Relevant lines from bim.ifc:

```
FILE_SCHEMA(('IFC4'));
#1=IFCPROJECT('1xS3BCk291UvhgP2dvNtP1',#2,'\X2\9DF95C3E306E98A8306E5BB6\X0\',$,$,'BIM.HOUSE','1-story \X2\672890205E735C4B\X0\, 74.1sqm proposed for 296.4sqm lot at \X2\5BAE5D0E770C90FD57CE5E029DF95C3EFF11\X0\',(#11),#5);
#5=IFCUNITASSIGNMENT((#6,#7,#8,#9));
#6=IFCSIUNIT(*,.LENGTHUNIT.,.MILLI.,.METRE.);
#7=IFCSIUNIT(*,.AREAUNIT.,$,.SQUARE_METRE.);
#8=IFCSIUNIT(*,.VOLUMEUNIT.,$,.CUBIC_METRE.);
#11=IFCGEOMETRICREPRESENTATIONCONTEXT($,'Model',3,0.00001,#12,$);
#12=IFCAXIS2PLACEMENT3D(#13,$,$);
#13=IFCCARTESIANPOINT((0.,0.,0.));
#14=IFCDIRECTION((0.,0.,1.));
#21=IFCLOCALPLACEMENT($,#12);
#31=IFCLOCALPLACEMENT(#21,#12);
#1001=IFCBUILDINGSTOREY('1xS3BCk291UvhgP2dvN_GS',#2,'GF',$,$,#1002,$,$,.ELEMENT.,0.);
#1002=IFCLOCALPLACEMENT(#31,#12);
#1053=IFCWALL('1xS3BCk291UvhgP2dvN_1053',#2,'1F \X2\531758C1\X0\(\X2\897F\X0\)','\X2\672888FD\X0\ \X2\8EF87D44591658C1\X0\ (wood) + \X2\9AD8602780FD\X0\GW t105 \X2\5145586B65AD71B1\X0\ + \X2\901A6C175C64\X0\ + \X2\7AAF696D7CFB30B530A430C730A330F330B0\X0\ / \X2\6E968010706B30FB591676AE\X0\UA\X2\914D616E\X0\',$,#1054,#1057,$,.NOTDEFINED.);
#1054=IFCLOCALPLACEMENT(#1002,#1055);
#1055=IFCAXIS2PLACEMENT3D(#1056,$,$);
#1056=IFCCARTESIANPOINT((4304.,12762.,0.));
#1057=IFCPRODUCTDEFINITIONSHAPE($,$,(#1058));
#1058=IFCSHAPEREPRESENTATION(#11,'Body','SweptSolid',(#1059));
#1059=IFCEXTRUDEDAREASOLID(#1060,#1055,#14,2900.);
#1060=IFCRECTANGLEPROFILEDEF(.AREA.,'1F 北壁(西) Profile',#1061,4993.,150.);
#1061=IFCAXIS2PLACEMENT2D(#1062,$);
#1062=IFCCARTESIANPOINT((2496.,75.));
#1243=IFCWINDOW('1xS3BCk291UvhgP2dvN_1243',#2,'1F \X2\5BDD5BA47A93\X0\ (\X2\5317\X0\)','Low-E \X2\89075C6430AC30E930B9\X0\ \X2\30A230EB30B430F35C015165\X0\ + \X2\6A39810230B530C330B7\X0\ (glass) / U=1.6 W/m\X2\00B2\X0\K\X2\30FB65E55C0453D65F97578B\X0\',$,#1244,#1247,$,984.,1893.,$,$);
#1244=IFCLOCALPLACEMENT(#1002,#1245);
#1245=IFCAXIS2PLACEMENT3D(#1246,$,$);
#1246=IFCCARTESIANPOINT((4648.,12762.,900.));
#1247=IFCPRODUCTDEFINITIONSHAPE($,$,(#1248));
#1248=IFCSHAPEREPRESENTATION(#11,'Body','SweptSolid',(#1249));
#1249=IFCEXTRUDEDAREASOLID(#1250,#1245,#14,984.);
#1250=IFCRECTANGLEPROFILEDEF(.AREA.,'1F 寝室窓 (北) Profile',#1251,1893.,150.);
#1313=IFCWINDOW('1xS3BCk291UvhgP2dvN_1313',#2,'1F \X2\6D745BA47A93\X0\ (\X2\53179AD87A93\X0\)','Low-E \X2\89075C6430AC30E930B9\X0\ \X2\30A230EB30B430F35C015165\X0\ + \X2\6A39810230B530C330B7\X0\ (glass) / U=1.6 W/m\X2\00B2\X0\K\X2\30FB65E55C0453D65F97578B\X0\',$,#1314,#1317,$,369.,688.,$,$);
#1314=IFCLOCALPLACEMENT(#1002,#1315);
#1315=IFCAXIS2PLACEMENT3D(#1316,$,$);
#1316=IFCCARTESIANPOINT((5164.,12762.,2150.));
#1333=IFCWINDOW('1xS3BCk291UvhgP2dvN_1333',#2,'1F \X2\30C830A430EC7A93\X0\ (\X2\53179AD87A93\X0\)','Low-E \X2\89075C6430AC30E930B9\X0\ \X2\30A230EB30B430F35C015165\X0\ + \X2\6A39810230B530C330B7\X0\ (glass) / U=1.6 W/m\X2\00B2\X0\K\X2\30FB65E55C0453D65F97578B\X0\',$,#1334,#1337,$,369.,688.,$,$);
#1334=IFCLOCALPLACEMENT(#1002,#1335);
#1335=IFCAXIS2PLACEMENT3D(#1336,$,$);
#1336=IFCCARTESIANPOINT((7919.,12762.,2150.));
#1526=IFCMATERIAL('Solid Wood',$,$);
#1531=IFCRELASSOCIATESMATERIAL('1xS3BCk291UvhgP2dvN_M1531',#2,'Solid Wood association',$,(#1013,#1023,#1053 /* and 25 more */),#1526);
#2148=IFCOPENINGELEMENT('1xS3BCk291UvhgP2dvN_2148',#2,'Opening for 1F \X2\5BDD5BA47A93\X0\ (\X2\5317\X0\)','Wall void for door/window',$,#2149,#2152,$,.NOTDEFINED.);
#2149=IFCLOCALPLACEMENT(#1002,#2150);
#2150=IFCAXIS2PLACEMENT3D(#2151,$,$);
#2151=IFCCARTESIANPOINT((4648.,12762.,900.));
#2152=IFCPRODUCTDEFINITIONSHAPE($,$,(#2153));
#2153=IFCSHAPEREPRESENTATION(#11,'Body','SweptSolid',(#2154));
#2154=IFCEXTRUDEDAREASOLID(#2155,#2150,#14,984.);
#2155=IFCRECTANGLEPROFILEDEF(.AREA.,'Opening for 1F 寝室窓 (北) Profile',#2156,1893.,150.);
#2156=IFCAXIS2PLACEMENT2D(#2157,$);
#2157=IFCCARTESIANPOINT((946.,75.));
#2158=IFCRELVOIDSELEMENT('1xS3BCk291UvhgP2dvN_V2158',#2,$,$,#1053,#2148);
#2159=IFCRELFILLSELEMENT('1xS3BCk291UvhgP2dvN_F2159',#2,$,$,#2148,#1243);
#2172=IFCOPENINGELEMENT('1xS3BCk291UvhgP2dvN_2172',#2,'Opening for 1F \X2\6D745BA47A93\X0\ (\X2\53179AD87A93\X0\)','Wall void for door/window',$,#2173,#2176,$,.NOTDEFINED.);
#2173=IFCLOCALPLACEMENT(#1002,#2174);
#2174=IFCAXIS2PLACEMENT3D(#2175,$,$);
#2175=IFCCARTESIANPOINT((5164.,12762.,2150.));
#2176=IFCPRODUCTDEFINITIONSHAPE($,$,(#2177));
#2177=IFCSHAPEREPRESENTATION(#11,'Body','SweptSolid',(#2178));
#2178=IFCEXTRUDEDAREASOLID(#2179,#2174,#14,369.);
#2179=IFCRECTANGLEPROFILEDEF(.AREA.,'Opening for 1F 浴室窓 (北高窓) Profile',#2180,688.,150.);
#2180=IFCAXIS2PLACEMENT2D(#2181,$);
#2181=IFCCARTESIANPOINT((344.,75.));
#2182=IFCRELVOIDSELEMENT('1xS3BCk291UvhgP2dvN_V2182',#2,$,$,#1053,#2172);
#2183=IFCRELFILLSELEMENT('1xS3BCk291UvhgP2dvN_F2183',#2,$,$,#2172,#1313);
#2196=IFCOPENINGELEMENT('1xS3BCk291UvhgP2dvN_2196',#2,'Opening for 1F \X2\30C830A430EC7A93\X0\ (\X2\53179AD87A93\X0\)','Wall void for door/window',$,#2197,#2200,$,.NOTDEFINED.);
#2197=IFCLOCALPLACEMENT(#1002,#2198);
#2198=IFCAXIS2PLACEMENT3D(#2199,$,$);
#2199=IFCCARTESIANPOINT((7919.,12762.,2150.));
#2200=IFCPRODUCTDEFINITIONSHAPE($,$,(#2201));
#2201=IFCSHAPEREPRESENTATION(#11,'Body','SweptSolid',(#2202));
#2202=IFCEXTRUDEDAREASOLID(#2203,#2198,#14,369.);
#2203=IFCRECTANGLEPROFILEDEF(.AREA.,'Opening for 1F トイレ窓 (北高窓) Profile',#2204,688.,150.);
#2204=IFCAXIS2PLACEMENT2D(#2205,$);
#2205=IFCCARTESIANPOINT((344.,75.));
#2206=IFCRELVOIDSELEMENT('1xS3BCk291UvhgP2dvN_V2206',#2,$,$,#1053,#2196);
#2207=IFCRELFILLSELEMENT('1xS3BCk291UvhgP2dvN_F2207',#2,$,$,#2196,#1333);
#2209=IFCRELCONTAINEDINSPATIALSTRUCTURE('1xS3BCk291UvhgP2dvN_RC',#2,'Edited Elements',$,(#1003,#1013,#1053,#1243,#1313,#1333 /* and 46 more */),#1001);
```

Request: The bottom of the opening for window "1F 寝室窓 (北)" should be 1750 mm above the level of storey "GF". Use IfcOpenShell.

```python
import numpy as np
import ifcopenshell
import ifcopenshell.api.geometry
import ifcopenshell.geom
import ifcopenshell.util.element
import ifcopenshell.util.placement
import ifcopenshell.util.shape
import ifcopenshell.util.unit

model = ifcopenshell.open("bim.ifc")
unit_scale = ifcopenshell.util.unit.calculate_unit_scale(model)

window = model.by_guid("1xS3BCk291UvhgP2dvN_1243")
opening = window.FillsVoids[0].RelatingOpeningElement
storey = ifcopenshell.util.element.get_container(window, ifc_class="IfcBuildingStorey")
level = ifcopenshell.util.placement.get_local_placement(storey.ObjectPlacement)[2, 3]

# The opening's origin need not be at the sill, so measure its lowest point.
shape = ifcopenshell.geom.create_shape(ifcopenshell.geom.settings(), opening)
bottom = ifcopenshell.util.shape.get_shape_bottom_elevation(shape, shape.geometry) / unit_scale
dz = level + 1.75 / unit_scale - bottom

shift = np.array([0.0, 0.0, dz])
# The window is not placed relative to its opening, so move both.
for product in (opening, window):
    matrix = ifcopenshell.util.placement.get_local_placement(product.ObjectPlacement)
    matrix[:3, 3] += shift
    ifcopenshell.api.geometry.edit_object_placement(model, product=product, matrix=matrix, is_si=False)

print(f"moved by {dz * unit_scale:+.3f} m")

model.write("bim_updated.ifc")
```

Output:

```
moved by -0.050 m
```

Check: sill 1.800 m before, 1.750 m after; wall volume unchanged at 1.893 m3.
